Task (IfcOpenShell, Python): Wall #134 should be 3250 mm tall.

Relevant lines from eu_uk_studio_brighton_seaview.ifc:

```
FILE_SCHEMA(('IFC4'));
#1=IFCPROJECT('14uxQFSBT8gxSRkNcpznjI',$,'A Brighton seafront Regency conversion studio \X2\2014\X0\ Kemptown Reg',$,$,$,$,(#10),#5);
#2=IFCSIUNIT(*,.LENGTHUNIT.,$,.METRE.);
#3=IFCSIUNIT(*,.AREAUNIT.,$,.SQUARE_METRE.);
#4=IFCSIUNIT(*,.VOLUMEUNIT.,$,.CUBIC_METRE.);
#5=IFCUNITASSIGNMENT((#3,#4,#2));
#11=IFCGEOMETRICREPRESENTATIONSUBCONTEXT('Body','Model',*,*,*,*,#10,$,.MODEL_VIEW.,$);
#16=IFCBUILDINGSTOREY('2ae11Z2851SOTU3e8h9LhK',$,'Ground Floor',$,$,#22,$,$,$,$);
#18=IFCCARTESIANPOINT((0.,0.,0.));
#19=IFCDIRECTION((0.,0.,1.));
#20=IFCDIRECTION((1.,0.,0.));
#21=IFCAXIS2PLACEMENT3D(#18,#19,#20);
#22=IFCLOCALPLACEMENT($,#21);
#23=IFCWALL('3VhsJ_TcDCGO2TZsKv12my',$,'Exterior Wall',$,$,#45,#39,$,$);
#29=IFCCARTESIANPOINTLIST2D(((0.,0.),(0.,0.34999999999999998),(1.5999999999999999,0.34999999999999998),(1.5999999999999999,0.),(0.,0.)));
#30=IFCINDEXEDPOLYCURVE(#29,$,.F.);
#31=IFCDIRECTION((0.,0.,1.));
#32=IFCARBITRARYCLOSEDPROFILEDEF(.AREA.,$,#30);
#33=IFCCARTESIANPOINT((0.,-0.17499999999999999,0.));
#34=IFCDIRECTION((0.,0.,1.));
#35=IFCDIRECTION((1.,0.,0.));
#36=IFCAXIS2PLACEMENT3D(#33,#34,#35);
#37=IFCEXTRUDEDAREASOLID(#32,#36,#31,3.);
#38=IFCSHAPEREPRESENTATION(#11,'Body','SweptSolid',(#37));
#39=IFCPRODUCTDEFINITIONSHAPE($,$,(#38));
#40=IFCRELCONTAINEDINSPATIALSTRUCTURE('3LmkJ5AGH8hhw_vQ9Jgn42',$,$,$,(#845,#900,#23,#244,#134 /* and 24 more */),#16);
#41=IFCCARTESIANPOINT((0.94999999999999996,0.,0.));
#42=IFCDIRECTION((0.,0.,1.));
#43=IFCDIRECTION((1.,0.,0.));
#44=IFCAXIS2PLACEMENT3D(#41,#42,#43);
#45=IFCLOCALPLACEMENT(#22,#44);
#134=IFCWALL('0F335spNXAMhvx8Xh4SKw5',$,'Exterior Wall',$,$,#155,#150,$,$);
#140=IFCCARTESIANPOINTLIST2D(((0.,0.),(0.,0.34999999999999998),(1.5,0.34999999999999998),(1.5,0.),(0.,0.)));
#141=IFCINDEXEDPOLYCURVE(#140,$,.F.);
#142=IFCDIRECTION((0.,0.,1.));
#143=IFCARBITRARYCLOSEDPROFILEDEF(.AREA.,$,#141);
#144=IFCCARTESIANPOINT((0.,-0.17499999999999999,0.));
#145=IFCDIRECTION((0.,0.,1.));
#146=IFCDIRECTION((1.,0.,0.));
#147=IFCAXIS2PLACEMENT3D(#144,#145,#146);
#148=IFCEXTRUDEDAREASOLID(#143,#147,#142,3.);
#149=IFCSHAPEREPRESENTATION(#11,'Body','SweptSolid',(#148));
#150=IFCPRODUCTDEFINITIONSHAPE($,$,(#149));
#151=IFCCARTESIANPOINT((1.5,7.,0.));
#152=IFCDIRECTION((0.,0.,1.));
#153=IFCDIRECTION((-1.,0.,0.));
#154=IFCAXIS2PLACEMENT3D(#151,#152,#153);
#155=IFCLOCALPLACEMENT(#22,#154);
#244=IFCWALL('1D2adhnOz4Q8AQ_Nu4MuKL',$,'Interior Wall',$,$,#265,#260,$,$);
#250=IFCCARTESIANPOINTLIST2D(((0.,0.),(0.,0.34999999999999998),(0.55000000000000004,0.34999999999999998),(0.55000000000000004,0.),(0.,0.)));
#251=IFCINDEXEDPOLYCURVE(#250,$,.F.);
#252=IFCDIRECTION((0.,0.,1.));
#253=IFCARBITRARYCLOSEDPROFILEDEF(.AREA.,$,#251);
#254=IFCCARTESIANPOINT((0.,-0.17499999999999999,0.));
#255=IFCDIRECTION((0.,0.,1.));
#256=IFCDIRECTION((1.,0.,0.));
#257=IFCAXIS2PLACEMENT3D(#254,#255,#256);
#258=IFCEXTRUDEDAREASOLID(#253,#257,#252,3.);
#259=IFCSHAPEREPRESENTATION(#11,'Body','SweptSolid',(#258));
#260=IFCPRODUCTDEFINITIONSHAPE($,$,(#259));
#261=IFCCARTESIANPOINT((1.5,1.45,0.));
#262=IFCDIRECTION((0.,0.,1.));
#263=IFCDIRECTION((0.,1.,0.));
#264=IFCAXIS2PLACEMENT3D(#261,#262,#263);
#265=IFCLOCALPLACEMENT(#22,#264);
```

```python
import ifcopenshell
import ifcopenshell.geom
import ifcopenshell.util.representation
import ifcopenshell.util.shape
import ifcopenshell.util.unit

model = ifcopenshell.open("eu_uk_studio_brighton_seaview.ifc")
unit_scale = ifcopenshell.util.unit.calculate_unit_scale(model)
settings = ifcopenshell.geom.settings()


def volume(element):
    """Net volume in cubic metres, openings subtracted."""
    shape = ifcopenshell.geom.create_shape(settings, element)
    return ifcopenshell.util.shape.get_volume(shape.geometry)


wall = model.by_guid("0F335spNXAMhvx8Xh4SKw5")
before = volume(wall)

body = ifcopenshell.util.representation.get_representation(wall, "Model", "Body")
solid = body.Items[0]
old_height = solid.Depth
solid.Depth = 3.25 / unit_scale
after = volume(wall)

print(f"height {old_height:g} -> {solid.Depth:g}, volume {before:.3f} -> {after:.3f} m3")

model.write("eu_uk_studio_brighton_seaview_edited.ifc")
```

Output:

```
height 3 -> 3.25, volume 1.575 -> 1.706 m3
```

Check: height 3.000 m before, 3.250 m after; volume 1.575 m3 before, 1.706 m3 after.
